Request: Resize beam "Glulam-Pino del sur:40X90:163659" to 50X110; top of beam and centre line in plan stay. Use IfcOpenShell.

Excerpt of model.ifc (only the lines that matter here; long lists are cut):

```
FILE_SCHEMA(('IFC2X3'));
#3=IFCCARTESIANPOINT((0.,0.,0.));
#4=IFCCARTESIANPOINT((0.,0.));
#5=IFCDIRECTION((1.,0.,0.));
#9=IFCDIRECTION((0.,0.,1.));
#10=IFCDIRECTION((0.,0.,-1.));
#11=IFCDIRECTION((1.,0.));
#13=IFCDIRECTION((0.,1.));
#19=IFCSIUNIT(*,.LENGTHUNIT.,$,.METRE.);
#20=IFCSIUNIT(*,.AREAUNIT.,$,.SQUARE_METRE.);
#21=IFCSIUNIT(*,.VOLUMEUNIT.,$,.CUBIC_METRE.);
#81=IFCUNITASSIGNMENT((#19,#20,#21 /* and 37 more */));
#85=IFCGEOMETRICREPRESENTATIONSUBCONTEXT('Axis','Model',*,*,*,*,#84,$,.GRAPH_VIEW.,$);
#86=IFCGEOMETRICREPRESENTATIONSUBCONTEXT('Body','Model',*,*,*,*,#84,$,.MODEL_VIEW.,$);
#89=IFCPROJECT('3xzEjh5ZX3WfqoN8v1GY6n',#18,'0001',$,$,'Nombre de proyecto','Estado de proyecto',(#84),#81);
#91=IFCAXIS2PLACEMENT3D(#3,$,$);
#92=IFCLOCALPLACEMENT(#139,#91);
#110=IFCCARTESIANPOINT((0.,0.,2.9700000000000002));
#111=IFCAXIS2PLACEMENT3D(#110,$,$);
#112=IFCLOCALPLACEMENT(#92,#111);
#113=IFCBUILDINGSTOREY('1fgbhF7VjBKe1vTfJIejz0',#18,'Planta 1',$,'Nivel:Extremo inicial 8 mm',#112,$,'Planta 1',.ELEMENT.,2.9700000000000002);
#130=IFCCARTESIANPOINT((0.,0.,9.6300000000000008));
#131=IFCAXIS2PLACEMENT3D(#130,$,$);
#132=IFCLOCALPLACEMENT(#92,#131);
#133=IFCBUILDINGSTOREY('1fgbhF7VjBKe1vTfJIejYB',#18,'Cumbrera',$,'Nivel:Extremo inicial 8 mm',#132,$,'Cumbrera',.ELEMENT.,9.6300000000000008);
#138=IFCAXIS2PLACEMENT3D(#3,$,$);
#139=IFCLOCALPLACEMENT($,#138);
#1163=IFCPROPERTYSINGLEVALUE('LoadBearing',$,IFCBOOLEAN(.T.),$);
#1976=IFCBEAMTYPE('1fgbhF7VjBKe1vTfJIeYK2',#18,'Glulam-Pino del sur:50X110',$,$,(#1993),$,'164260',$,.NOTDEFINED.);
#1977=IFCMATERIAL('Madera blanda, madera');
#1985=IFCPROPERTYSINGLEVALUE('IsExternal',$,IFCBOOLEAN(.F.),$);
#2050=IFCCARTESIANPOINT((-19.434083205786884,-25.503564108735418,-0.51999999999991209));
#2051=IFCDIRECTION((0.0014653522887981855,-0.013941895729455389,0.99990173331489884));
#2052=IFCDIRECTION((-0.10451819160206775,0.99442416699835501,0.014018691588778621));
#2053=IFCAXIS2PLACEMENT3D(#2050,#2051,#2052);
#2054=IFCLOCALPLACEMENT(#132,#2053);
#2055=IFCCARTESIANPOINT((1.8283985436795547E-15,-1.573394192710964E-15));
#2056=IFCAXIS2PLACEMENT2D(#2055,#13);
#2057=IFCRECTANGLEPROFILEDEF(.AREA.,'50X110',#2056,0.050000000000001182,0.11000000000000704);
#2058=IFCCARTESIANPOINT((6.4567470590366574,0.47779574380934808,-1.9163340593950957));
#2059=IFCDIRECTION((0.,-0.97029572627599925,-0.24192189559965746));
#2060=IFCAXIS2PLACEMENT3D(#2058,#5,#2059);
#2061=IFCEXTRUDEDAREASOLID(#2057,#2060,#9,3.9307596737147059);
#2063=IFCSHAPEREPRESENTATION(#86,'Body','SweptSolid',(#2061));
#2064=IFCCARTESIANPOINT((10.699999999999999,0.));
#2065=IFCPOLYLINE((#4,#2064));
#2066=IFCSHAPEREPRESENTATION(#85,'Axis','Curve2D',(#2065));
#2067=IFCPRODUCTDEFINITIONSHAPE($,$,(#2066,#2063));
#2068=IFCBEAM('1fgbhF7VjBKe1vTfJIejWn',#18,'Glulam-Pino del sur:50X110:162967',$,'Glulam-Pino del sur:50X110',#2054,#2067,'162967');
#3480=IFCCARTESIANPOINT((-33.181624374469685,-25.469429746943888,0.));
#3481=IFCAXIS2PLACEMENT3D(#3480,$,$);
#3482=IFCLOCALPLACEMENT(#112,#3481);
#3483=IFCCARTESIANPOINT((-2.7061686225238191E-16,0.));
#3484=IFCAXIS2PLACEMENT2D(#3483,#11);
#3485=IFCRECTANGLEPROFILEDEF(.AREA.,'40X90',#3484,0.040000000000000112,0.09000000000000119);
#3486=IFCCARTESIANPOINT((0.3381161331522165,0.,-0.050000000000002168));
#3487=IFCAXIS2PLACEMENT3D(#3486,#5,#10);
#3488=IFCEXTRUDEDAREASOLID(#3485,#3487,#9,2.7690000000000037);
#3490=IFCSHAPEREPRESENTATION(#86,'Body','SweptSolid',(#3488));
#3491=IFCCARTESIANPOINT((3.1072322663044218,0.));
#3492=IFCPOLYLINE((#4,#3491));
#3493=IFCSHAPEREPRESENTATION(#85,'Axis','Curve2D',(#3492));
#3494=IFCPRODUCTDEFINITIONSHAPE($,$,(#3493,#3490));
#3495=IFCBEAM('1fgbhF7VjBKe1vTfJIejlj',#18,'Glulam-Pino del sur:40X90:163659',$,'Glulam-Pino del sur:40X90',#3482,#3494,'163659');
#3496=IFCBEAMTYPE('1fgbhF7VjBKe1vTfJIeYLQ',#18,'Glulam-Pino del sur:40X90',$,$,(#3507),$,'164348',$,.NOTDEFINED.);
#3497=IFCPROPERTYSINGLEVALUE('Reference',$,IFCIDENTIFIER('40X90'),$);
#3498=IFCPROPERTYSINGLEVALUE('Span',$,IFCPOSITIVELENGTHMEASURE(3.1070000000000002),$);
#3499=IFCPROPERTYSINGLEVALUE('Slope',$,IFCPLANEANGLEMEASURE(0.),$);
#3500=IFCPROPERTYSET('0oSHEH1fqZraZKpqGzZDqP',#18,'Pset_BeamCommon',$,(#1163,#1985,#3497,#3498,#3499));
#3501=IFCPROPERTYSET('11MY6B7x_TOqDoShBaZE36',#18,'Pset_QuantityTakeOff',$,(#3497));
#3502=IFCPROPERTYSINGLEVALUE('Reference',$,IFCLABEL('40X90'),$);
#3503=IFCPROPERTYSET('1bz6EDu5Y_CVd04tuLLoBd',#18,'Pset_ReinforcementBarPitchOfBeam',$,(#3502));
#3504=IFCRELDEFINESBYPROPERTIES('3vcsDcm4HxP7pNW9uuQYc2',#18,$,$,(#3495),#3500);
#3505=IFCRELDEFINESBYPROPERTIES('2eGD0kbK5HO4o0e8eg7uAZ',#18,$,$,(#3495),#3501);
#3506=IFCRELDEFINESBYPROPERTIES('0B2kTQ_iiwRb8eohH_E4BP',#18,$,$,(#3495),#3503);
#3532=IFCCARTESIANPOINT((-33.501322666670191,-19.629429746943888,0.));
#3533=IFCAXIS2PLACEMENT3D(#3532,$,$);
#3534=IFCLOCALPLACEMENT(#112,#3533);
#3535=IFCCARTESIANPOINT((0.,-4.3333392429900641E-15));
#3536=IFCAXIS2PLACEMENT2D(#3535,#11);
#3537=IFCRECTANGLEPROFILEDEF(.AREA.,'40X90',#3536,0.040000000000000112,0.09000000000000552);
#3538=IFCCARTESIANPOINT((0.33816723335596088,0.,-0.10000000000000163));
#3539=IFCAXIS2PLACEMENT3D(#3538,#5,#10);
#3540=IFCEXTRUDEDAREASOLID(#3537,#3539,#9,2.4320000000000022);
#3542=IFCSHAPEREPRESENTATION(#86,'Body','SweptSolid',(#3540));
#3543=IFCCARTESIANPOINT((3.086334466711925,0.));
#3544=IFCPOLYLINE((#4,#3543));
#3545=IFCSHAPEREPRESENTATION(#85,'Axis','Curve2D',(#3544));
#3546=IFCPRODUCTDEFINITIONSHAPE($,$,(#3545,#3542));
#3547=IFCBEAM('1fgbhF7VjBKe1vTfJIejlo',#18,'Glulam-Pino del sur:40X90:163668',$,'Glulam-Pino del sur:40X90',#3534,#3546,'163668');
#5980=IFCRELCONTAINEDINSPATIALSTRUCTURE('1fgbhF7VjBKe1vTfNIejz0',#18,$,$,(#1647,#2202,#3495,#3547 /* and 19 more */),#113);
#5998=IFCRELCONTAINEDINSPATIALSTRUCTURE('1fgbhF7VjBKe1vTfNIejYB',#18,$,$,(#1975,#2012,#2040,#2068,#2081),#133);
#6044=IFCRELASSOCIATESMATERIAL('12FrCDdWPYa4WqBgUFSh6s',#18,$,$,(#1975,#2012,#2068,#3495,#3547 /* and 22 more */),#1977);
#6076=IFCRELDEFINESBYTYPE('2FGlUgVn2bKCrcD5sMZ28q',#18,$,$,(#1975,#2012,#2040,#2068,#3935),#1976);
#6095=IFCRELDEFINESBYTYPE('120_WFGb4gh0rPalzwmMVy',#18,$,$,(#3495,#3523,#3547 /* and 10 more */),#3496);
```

```python
import ifcopenshell
import ifcopenshell.api.pset
import ifcopenshell.api.type
import ifcopenshell.util.element
import ifcopenshell.util.representation

model = ifcopenshell.open("model.ifc")

member = model.by_guid("1fgbhF7VjBKe1vTfJIejlj")
source = next(p for p in model.by_type("IfcRectangleProfileDef") if p.ProfileName == "50X110")

body = ifcopenshell.util.representation.get_representation(member, "Model", "Body")
solid = body.Items[0]
old_profile = solid.SweptArea

# Copy the section's sizes but keep this member's own profile position.
profile = ifcopenshell.util.element.copy(model, source)
# Profiles are centred, so shift by half the change in depth to hold the top.
shift = (old_profile.XDim - profile.XDim) / 2
x, y = old_profile.Position.Location.Coordinates
up = (-1.0, 0.0)  # upwards, in the solid's own plane
location = model.createIfcCartesianPoint((x + up[0] * shift, y + up[1] * shift))
profile.Position = model.createIfcAxis2Placement2D(location, old_profile.Position.RefDirection)
solid.SweptArea = profile
if not model.get_total_inverses(old_profile):
    ifcopenshell.util.element.remove_deep2(model, old_profile)

new_type = model.by_guid("1fgbhF7VjBKe1vTfJIeYK2")
ifcopenshell.api.type.assign_type(
    model, related_objects=[member], relating_type=new_type, should_map_representations=False
)
member.Name = member.Name.replace("40X90", "50X110")
member.ObjectType = "Glulam-Pino del sur:50X110"
pset = model.by_id(ifcopenshell.util.element.get_pset(member, "Pset_BeamCommon", should_inherit=False)["id"])
ifcopenshell.api.pset.edit_pset(model, pset=pset, properties={"Reference": "50X110"})
pset = model.by_id(ifcopenshell.util.element.get_pset(member, "Pset_QuantityTakeOff", should_inherit=False)["id"])
ifcopenshell.api.pset.edit_pset(model, pset=pset, properties={"Reference": "50X110"})
pset = model.by_id(ifcopenshell.util.element.get_pset(member, "Pset_ReinforcementBarPitchOfBeam", should_inherit=False)["id"])
ifcopenshell.api.pset.edit_pset(model, pset=pset, properties={"Reference": "50X110"})

print(solid.SweptArea)

model.write("model_v2.ifc")
```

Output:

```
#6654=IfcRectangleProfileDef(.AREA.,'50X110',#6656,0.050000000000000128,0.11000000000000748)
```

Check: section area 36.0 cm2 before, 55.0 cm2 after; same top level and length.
